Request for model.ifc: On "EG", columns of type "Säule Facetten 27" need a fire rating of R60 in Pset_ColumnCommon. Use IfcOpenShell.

First a look at what the model holds.

```python
import ifcopenshell
import ifcopenshell.util.element

model = ifcopenshell.open("model.ifc")
print(model.schema)
storey = next(s for s in model.by_type("IfcBuildingStorey") if s.Name == "EG")
columns = [e for e in ifcopenshell.util.element.get_decomposition(storey) if e.is_a("IfcColumn")]
seen = {}
for e in columns:
    element_type = ifcopenshell.util.element.get_type(e)
    key = (element_type.Name if element_type != e and element_type else None, ifcopenshell.util.element.get_pset(e, "Pset_ColumnCommon", "FireRating"))
    seen[key] = seen.get(key, 0) + 1
for (name, value), count in sorted(seen.items(), key=str):
    print(count, "x", name, "|", value)
```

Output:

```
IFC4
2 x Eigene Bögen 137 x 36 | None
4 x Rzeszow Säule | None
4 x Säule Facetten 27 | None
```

```python
import ifcopenshell
import ifcopenshell.api.pset
import ifcopenshell.util.element

model = ifcopenshell.open("model.ifc")

storey = next(s for s in model.by_type("IfcBuildingStorey") if s.Name == "EG")
columns = [e for e in ifcopenshell.util.element.get_decomposition(storey) if e.is_a("IfcColumn")]

count = 0
for e in columns:
    element_type = ifcopenshell.util.element.get_type(e)
    if element_type in (None, e) or element_type.Name != "Säule Facetten 27":
        continue
    # add_pset returns the element's existing set when there is one.
    pset = ifcopenshell.api.pset.add_pset(model, product=e, name="Pset_ColumnCommon")
    ifcopenshell.api.pset.edit_pset(model, pset=pset, properties={"FireRating": "R60"})
    count += 1

print(count, "columns updated")

model.write("model_updated.ifc")
```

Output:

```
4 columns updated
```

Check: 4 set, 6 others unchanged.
